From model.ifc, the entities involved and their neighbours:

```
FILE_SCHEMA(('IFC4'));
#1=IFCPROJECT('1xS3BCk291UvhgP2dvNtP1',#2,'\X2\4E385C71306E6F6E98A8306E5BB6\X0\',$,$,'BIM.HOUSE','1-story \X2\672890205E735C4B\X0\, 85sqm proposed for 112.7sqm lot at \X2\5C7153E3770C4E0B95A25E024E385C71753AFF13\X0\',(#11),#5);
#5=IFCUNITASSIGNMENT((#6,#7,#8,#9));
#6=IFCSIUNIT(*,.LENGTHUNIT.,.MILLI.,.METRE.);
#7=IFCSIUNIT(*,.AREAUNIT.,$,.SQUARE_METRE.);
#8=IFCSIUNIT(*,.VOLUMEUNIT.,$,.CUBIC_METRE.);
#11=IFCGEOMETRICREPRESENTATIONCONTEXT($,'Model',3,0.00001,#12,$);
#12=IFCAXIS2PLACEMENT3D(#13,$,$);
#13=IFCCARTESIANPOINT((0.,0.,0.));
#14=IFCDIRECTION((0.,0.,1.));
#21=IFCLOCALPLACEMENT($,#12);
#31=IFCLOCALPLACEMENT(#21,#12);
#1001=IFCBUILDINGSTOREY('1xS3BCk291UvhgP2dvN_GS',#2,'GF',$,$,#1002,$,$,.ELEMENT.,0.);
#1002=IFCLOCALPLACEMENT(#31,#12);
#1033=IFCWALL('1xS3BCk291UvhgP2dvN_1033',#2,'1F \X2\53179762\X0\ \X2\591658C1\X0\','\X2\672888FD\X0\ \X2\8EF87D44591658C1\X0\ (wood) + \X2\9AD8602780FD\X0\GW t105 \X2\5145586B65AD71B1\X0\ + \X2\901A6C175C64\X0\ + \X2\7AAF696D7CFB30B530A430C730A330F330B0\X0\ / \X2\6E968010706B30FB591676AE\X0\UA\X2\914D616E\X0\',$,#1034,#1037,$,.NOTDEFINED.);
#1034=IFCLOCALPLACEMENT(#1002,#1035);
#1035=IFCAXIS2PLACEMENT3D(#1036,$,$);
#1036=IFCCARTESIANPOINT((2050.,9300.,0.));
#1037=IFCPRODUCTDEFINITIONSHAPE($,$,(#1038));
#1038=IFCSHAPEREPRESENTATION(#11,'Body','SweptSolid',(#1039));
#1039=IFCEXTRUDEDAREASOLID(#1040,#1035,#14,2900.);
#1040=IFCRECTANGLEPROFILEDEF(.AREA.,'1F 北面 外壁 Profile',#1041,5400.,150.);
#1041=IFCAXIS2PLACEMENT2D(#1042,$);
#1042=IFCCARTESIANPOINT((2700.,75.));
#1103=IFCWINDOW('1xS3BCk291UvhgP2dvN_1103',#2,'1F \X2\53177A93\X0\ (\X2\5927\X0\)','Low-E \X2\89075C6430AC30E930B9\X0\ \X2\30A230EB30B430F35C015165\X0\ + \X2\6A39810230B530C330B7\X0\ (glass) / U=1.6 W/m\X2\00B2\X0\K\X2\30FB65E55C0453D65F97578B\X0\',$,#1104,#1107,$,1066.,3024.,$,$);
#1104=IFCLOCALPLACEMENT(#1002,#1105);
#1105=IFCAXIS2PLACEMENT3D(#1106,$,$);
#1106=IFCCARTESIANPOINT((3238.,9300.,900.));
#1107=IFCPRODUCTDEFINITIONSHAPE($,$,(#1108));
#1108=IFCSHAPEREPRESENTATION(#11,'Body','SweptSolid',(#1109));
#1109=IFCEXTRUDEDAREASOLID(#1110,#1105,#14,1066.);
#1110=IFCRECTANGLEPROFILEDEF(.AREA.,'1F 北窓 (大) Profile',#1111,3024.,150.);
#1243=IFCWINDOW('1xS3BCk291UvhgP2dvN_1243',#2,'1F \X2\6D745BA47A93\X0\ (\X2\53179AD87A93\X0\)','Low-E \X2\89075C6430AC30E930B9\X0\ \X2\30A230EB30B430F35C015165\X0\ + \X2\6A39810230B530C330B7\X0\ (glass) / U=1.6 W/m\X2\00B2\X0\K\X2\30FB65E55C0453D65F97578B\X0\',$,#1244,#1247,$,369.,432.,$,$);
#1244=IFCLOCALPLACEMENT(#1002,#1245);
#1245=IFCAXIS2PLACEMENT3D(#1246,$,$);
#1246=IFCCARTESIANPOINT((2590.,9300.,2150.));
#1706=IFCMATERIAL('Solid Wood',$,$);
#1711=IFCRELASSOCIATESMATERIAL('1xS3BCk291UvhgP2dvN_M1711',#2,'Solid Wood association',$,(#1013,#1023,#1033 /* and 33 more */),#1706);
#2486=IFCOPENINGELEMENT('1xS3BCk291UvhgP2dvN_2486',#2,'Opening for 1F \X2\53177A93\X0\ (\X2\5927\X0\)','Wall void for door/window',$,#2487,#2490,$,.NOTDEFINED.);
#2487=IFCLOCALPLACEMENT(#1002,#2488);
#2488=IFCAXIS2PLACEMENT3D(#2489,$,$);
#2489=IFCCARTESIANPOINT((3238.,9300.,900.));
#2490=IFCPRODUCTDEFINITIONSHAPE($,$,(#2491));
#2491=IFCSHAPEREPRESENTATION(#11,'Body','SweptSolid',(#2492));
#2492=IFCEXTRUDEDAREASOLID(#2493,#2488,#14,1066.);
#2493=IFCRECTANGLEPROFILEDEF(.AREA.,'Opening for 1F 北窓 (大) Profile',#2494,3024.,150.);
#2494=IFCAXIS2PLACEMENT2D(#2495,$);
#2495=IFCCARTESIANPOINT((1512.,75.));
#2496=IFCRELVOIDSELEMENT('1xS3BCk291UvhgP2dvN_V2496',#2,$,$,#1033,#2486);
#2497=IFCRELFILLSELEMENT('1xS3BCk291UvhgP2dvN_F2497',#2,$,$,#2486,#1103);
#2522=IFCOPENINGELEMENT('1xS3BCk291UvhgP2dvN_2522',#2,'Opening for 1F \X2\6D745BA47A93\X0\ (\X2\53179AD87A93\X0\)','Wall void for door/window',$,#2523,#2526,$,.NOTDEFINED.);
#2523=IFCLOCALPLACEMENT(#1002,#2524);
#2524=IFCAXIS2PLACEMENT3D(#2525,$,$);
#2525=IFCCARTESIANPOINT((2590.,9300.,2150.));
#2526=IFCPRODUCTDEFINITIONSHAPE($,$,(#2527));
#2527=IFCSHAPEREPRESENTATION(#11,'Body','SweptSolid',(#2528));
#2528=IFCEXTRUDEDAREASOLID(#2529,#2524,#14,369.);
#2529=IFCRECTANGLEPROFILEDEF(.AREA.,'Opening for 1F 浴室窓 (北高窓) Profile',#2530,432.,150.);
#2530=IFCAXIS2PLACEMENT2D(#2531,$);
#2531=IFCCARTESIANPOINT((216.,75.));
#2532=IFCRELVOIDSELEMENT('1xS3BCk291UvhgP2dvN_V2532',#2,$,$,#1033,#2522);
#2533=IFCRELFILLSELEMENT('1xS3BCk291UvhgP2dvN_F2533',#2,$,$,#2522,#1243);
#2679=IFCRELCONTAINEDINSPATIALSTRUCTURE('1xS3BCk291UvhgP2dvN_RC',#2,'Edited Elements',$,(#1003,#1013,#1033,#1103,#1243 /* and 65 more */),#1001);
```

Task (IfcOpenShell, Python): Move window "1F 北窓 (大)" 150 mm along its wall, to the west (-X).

```python
import ifcopenshell
import ifcopenshell.api.geometry
import ifcopenshell.util.placement
import ifcopenshell.util.unit

model = ifcopenshell.open("model.ifc")
unit_scale = ifcopenshell.util.unit.calculate_unit_scale(model)

window = model.by_guid("1xS3BCk291UvhgP2dvN_1103")
opening = window.FillsVoids[0].RelatingOpeningElement
wall = opening.VoidsElements[0].RelatingBuildingElement

wall_matrix = ifcopenshell.util.placement.get_local_placement(wall.ObjectPlacement)
shift = wall_matrix[:3, 0] * -0.15 / unit_scale
before = ifcopenshell.util.placement.get_local_placement(window.ObjectPlacement)[:3, 3].copy()

# The window is not placed relative to its opening, so move both.
for product in (opening, window):
    matrix = ifcopenshell.util.placement.get_local_placement(product.ObjectPlacement)
    matrix[:3, 3] += shift
    ifcopenshell.api.geometry.edit_object_placement(model, product=product, matrix=matrix, is_si=False)

after = ifcopenshell.util.placement.get_local_placement(window.ObjectPlacement)[:3, 3]
print("window moved by", (after - before).round(3) + 0.0)

model.write("model_rev.ifc")
```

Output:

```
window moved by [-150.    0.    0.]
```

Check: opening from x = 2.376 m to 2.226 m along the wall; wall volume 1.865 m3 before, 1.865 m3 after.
